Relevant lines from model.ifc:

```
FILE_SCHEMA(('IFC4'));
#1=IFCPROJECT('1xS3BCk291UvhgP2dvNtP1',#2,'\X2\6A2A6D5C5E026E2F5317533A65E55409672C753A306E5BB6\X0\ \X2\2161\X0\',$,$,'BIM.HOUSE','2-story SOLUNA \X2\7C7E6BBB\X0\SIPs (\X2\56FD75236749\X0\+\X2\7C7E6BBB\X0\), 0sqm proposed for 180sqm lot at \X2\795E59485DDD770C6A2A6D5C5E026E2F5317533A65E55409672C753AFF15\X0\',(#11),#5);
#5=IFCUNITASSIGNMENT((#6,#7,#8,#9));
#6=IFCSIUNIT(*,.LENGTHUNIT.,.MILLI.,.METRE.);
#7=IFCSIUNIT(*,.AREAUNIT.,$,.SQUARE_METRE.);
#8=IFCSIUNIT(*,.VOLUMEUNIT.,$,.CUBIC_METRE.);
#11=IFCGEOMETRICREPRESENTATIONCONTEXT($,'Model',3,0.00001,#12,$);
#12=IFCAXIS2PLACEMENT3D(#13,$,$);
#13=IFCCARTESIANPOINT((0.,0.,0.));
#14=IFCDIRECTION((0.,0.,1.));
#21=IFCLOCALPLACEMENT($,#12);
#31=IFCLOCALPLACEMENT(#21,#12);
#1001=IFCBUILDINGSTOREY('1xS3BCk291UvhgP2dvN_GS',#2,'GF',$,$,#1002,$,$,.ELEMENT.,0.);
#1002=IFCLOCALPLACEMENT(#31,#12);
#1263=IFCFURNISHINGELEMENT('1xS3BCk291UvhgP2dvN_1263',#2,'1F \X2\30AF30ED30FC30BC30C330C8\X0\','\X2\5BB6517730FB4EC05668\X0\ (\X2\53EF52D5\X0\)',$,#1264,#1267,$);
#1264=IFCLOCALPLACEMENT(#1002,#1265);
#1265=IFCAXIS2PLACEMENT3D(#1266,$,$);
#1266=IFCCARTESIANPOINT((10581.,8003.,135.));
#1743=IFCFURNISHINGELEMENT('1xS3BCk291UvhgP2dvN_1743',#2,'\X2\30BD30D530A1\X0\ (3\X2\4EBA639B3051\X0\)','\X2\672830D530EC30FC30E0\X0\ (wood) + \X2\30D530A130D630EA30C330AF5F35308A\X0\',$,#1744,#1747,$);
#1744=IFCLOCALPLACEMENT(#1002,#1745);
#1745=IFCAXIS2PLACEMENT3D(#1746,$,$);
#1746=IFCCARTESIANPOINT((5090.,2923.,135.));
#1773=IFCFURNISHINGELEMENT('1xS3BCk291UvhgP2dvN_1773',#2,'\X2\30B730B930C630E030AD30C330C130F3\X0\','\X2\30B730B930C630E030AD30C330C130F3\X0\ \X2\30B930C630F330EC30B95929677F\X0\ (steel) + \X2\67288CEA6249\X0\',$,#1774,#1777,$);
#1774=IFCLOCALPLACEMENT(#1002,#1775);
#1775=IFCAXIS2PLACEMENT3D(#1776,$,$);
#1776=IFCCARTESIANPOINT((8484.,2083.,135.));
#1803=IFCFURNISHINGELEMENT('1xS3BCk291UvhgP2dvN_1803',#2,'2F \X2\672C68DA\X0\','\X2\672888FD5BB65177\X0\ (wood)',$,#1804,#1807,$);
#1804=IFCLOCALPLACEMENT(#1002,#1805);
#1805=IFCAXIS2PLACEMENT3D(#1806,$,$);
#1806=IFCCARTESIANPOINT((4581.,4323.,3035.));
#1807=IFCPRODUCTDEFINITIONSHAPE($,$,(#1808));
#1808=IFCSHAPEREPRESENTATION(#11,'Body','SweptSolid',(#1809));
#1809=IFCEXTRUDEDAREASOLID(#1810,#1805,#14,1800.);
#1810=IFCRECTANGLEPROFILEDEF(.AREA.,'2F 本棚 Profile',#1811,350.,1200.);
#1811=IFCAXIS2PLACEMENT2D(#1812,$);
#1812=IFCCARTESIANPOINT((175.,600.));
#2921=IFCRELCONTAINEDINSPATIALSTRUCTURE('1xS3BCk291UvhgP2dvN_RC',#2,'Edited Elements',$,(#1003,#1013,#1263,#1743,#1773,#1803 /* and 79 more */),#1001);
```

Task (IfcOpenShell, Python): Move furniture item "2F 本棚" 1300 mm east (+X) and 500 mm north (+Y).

```python
import ifcopenshell
import ifcopenshell.api.geometry
import ifcopenshell.util.placement
import ifcopenshell.util.unit

model = ifcopenshell.open("model.ifc")
unit_scale = ifcopenshell.util.unit.calculate_unit_scale(model)

item = model.by_id(1803)
matrix = ifcopenshell.util.placement.get_local_placement(item.ObjectPlacement)
matrix[0, 3] += 1.3 / unit_scale
matrix[1, 3] += 0.5 / unit_scale
ifcopenshell.api.geometry.edit_object_placement(model, product=item, matrix=matrix, is_si=False)

print(ifcopenshell.util.placement.get_local_placement(item.ObjectPlacement).round(3) + 0.0)

model.write("model_edited.ifc")
```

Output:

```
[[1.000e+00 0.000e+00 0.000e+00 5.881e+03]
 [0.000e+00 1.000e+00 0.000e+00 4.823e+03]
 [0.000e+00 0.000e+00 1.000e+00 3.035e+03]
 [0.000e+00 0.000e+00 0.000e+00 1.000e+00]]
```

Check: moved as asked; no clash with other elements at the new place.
